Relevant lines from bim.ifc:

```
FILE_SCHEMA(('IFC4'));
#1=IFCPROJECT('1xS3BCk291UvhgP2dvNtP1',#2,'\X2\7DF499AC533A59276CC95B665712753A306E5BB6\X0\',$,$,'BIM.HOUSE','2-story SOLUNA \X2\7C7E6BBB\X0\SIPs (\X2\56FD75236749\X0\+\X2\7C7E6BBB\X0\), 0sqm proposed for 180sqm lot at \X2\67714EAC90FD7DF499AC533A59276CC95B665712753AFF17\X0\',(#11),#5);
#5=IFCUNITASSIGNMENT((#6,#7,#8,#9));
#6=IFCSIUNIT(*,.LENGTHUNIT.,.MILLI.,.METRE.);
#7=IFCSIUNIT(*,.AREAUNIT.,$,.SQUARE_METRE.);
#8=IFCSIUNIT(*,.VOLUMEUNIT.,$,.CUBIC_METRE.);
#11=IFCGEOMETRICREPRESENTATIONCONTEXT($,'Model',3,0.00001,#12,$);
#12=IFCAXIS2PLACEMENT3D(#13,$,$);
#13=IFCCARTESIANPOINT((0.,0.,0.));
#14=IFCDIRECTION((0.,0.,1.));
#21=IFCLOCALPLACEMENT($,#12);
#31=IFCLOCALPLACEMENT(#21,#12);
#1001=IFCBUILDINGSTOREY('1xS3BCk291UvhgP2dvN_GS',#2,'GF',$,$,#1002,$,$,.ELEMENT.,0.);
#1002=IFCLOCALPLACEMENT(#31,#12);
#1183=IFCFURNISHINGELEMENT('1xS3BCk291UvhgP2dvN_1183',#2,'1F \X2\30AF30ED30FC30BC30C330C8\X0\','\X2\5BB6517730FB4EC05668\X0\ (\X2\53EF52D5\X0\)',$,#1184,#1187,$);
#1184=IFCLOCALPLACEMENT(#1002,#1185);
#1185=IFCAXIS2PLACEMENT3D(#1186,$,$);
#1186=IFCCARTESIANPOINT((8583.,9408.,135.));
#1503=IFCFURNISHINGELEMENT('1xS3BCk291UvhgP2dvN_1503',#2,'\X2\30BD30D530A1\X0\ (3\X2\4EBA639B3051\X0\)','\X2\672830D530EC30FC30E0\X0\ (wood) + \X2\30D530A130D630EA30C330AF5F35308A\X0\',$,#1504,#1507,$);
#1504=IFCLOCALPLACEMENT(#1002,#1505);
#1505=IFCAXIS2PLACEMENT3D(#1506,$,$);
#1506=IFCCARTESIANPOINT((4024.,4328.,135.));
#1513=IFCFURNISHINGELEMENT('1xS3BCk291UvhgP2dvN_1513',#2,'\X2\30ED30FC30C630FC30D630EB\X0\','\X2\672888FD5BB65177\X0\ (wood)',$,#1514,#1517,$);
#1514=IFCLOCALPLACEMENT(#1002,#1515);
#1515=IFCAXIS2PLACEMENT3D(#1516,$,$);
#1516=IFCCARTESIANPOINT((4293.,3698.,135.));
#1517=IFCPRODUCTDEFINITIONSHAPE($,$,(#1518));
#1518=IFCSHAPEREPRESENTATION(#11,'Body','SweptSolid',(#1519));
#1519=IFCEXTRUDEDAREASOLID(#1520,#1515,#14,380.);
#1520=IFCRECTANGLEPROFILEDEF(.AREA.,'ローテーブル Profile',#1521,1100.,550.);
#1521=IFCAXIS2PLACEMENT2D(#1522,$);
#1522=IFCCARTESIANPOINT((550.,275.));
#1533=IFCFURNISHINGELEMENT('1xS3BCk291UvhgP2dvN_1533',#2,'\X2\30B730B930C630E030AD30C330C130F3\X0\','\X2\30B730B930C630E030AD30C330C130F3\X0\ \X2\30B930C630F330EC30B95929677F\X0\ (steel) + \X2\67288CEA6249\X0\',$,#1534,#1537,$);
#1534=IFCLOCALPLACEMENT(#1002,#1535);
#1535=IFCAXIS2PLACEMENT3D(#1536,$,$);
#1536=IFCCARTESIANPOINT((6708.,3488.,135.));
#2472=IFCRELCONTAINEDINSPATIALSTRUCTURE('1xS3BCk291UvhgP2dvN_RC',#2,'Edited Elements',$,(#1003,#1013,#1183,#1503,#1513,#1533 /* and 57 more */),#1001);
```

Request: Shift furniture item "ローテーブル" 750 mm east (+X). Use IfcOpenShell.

```python
import ifcopenshell
import ifcopenshell.api.geometry
import ifcopenshell.util.placement

model = ifcopenshell.open("bim.ifc")

item = model.by_guid("1xS3BCk291UvhgP2dvN_1513")
matrix = ifcopenshell.util.placement.get_local_placement(item.ObjectPlacement)
matrix[0, 3] += 750.0
ifcopenshell.api.geometry.edit_object_placement(model, product=item, matrix=matrix, is_si=False)

print(ifcopenshell.util.placement.get_local_placement(item.ObjectPlacement).round(3) + 0.0)

model.write("bim_updated.ifc")
```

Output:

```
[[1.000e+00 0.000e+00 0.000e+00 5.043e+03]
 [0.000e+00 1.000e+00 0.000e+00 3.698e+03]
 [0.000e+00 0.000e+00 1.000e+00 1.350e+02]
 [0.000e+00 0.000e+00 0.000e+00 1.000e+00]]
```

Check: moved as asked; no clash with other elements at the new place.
